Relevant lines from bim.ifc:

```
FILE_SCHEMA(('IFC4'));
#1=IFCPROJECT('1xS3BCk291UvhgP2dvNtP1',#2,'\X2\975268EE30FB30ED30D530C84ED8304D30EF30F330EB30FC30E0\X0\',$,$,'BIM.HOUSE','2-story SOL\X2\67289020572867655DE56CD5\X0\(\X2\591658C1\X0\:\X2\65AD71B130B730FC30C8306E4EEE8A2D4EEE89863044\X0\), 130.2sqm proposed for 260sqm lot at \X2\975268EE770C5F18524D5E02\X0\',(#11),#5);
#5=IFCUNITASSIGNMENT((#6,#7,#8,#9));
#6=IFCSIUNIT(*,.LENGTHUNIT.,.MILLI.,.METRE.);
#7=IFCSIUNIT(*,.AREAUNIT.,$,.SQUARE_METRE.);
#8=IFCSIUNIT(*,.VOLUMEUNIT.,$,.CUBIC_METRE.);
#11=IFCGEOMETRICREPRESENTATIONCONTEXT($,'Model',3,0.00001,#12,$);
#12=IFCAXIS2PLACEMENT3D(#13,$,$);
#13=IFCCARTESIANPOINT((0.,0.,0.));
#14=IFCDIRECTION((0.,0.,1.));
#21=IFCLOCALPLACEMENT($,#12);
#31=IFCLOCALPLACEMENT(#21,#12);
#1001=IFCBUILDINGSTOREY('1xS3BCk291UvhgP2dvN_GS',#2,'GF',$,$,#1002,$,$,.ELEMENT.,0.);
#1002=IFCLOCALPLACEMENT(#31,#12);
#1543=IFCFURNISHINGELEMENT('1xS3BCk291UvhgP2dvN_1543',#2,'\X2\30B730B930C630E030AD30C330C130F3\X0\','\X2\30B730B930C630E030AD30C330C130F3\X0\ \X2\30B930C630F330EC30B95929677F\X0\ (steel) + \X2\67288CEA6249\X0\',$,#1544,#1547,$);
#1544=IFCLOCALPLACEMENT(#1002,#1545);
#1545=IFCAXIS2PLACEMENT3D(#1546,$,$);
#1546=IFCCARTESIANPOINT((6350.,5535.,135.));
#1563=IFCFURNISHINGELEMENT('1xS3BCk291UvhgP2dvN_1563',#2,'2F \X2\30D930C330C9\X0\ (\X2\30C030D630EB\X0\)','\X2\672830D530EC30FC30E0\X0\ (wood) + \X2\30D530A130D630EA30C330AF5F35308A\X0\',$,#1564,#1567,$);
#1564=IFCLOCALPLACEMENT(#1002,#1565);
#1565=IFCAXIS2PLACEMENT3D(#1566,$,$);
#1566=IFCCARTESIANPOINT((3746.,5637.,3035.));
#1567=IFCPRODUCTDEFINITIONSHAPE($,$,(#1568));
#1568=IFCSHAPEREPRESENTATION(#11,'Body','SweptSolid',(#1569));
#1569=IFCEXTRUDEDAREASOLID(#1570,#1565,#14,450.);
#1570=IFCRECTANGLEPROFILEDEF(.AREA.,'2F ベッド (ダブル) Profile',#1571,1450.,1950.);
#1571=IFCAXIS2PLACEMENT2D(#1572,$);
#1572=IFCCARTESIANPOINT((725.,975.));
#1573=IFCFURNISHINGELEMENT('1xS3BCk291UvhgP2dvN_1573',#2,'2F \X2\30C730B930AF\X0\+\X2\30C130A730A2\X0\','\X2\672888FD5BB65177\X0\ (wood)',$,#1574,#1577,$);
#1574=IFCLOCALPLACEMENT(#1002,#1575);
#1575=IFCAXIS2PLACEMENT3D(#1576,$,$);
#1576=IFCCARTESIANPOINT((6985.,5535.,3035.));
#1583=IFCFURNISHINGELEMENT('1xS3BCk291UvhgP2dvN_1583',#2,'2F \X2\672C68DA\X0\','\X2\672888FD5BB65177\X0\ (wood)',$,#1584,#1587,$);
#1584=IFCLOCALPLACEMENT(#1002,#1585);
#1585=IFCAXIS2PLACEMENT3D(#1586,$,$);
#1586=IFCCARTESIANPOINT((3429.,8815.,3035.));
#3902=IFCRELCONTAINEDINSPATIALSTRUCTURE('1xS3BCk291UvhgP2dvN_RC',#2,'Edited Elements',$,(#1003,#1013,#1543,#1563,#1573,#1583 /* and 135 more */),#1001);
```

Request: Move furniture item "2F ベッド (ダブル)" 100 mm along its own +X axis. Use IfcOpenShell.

```python
import ifcopenshell
import ifcopenshell.api.geometry
import ifcopenshell.util.placement
import ifcopenshell.util.unit

model = ifcopenshell.open("bim.ifc")
unit_scale = ifcopenshell.util.unit.calculate_unit_scale(model)

item = model.by_id(1563)
matrix = ifcopenshell.util.placement.get_local_placement(item.ObjectPlacement)
matrix[:3, 3] += matrix[:3, 0] * 0.1 / unit_scale
ifcopenshell.api.geometry.edit_object_placement(model, product=item, matrix=matrix, is_si=False)

print(ifcopenshell.util.placement.get_local_placement(item.ObjectPlacement).round(3) + 0.0)

model.write("bim_rev.ifc")
```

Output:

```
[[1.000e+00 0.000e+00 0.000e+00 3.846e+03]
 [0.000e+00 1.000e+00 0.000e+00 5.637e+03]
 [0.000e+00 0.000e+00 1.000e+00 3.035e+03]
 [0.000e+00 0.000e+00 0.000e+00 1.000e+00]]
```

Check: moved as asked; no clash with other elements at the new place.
